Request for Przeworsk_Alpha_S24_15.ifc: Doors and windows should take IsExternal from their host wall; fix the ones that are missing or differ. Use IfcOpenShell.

First a look at what the model holds.

```python
import ifcopenshell
import ifcopenshell.util.element

model = ifcopenshell.open("Przeworsk_Alpha_S24_15.ifc")
print(model.schema)
seen = {}
for e in model.by_type("IfcDoor") + model.by_type("IfcWindow"):
    if not e.FillsVoids:
        continue
    host = e.FillsVoids[0].RelatingOpeningElement.VoidsElements[0].RelatingBuildingElement
    own = ifcopenshell.util.element.get_pset(e, f"Pset_{e.is_a()[3:].removesuffix('StandardCase')}Common", "IsExternal")
    wall = ifcopenshell.util.element.get_pset(host, "Pset_WallCommon", "IsExternal")
    seen[e.is_a(), own, wall] = seen.get((e.is_a(), own, wall), 0) + 1
for (cls, own, wall), count in sorted(seen.items(), key=str):
    print(count, cls, "IsExternal:", own, "| host wall:", wall)
```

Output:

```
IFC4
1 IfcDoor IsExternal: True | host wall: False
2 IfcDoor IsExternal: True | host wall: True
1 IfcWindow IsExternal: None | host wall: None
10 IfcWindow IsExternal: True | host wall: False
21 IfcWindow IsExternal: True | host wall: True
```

```python
import ifcopenshell
import ifcopenshell.api.pset
import ifcopenshell.util.element

model = ifcopenshell.open("Przeworsk_Alpha_S24_15.ifc")

count = 0
for ifc_class, pset_name in (("IfcDoor", "Pset_DoorCommon"), ("IfcWindow", "Pset_WindowCommon")):
    for e in model.by_type(ifc_class):
        if not e.FillsVoids:
            continue
        host = e.FillsVoids[0].RelatingOpeningElement.VoidsElements[0].RelatingBuildingElement
        external = ifcopenshell.util.element.get_pset(host, "Pset_WallCommon", "IsExternal")
        if external is None or ifcopenshell.util.element.get_pset(e, pset_name, "IsExternal") == external:
            continue
        pset = ifcopenshell.api.pset.add_pset(model, product=e, name=pset_name)
        ifcopenshell.api.pset.edit_pset(model, pset=pset, properties={"IsExternal": external})
        count += 1

print(count, "updated")

model.write("Przeworsk_Alpha_S24_15-out.ifc")
```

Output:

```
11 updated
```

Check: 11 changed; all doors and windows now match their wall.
